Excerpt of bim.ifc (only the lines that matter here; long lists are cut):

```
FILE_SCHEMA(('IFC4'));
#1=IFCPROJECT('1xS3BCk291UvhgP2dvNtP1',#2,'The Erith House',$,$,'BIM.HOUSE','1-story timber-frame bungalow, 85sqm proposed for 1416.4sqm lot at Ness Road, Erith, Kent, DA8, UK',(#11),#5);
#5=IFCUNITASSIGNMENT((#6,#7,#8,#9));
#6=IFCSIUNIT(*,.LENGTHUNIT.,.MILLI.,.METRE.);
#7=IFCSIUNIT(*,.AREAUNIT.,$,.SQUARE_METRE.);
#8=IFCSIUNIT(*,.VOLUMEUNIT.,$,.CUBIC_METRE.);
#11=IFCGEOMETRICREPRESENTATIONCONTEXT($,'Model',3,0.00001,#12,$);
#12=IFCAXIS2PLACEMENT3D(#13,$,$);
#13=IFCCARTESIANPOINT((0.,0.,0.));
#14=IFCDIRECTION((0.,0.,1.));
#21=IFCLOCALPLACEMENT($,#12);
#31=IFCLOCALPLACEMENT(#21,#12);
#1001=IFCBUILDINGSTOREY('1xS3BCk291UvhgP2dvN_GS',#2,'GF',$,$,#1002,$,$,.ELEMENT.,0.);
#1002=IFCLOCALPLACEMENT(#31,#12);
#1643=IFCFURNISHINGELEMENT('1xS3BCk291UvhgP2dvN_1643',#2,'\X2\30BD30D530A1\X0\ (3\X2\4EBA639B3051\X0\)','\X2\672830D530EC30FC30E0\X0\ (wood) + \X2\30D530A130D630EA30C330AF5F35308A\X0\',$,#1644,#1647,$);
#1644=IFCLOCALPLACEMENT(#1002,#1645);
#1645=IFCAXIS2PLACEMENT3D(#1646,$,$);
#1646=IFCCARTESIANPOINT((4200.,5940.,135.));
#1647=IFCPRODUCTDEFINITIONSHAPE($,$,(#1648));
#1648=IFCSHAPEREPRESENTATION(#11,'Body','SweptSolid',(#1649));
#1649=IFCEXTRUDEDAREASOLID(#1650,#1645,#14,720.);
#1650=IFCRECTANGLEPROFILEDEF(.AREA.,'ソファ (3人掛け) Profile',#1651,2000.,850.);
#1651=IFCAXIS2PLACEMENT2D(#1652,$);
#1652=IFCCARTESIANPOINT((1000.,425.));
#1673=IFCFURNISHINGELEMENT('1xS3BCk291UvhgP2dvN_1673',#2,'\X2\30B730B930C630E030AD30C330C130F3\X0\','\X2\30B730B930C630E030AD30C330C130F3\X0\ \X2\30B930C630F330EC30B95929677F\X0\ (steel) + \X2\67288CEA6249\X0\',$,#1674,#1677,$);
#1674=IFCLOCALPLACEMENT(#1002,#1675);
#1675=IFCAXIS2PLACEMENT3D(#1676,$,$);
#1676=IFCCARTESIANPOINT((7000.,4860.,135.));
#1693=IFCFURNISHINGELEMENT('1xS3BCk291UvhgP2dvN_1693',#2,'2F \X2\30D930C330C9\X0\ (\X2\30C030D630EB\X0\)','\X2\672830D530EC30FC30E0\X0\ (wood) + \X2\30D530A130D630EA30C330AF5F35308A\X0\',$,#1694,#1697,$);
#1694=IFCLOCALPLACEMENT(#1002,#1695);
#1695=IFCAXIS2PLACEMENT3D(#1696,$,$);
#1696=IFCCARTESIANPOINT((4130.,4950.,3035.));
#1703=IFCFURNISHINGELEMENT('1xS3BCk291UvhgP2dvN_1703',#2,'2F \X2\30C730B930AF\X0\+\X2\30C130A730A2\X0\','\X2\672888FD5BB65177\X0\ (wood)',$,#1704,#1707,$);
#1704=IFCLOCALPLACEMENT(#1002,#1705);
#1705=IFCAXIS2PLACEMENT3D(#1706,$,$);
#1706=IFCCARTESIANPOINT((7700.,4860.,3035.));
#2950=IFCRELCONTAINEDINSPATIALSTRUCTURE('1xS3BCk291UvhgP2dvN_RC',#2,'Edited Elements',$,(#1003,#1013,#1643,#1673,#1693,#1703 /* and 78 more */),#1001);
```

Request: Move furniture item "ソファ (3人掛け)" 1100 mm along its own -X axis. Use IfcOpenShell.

```python
import ifcopenshell
import ifcopenshell.api.geometry
import ifcopenshell.util.placement

model = ifcopenshell.open("bim.ifc")

item = model.by_guid("1xS3BCk291UvhgP2dvN_1643")
matrix = ifcopenshell.util.placement.get_local_placement(item.ObjectPlacement)
matrix[:3, 3] -= matrix[:3, 0] * 1100.0
ifcopenshell.api.geometry.edit_object_placement(model, product=item, matrix=matrix, is_si=False)

print(ifcopenshell.util.placement.get_local_placement(item.ObjectPlacement).round(3) + 0.0)

model.write("bim_v2.ifc")
```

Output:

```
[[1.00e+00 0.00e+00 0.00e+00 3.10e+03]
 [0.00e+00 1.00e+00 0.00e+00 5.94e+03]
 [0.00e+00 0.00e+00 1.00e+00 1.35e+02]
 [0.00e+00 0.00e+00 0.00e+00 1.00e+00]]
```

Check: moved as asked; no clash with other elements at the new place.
